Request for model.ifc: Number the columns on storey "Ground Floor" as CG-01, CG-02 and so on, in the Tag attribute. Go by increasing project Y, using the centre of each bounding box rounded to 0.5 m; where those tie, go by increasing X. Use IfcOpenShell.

First a look at what the model holds.

```python
import ifcopenshell
import ifcopenshell.util.element
import ifcopenshell.util.placement

model = ifcopenshell.open("model.ifc")
print(model.schema)
storey = next(s for s in model.by_type("IfcBuildingStorey") if s.Name == "Ground Floor")
columns = [e for e in ifcopenshell.util.element.get_decomposition(storey) if e.is_a("IfcColumn")]
for e in sorted(columns, key=lambda e: e.id()):
    origin = ifcopenshell.util.placement.get_local_placement(e.ObjectPlacement)[:3, 3]
    print(e.id(), e.Tag, e.Name, origin.round(2) + 0.0, sep=" | ")
```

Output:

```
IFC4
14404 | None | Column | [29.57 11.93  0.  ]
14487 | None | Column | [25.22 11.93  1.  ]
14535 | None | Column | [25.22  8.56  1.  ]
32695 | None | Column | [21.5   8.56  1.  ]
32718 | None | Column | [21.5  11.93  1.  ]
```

```python
import ifcopenshell
import ifcopenshell.geom
import ifcopenshell.util.element
import ifcopenshell.util.shape

model = ifcopenshell.open("model.ifc")
settings = ifcopenshell.geom.settings()
settings.set("use-world-coords", True)


def centre(element):
    shape = ifcopenshell.geom.create_shape(settings, element)
    return ifcopenshell.util.shape.get_bbox_centroid(shape.geometry)


storey = next(s for s in model.by_type("IfcBuildingStorey") if s.Name == "Ground Floor")
columns = [e for e in ifcopenshell.util.element.get_decomposition(storey) if e.is_a("IfcColumn")]

# Insertion points can sit at a corner or the storey origin, so sort by the geometry (in metres).
centres = {e: centre(e) for e in columns}
columns.sort(key=lambda e: (round(centres[e][1] / 0.5), centres[e][0]))

for i, e in enumerate(columns, start=1):
    number = f"CG-{i:02d}"
    e.Tag = number
    print(e.id(), number)

model.write("model-out.ifc")
```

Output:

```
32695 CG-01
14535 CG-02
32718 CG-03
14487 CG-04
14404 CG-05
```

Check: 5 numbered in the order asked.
